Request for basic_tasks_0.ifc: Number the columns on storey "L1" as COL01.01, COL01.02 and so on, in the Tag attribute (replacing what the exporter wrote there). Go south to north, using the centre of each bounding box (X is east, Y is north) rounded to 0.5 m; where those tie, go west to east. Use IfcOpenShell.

First a look at what the model holds.

```python
import ifcopenshell
import ifcopenshell.util.element
import ifcopenshell.util.placement

model = ifcopenshell.open("basic_tasks_0.ifc")
print(model.schema)
storey = next(s for s in model.by_type("IfcBuildingStorey") if s.Name == "L1")
columns = [e for e in ifcopenshell.util.element.get_decomposition(storey) if e.is_a("IfcColumn")]
for e in sorted(columns, key=lambda e: e.id()):
    origin = ifcopenshell.util.placement.get_local_placement(e.ObjectPlacement)[:3, 3]
    print(e.id(), e.Tag, e.Name, origin.round(2) + 0.0, sep=" | ")
```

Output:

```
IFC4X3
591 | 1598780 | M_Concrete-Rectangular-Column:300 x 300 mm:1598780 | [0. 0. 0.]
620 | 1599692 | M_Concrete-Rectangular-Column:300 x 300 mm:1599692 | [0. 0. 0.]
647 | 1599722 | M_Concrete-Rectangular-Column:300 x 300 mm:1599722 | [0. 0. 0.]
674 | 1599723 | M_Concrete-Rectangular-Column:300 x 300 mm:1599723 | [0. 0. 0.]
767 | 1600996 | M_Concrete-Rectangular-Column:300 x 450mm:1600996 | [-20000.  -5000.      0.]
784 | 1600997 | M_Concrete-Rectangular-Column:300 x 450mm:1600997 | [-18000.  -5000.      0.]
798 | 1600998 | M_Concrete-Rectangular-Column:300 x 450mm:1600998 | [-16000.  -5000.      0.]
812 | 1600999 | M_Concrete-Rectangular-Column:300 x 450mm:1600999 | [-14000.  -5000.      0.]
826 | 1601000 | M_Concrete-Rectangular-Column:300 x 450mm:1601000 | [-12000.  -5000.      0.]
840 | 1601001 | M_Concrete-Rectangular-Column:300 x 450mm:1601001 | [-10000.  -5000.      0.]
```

```python
import ifcopenshell
import ifcopenshell.geom
import ifcopenshell.util.element
import ifcopenshell.util.shape

model = ifcopenshell.open("basic_tasks_0.ifc")
settings = ifcopenshell.geom.settings()
settings.set("use-world-coords", True)


def centre(element):
    shape = ifcopenshell.geom.create_shape(settings, element)
    return ifcopenshell.util.shape.get_bbox_centroid(shape.geometry)


storey = next(s for s in model.by_type("IfcBuildingStorey") if s.Name == "L1")
columns = [e for e in ifcopenshell.util.element.get_decomposition(storey) if e.is_a("IfcColumn")]

# Insertion points can sit at a corner or the storey origin, so sort by the geometry (in metres).
centres = {e: centre(e) for e in columns}
columns.sort(key=lambda e: (round(centres[e][1] / 0.5), centres[e][0]))

for i, e in enumerate(columns, start=1):
    number = f"COL01.{i:02d}"
    e.Tag = number
    print(e.id(), number)

model.write("basic_tasks_0_updated.ifc")
```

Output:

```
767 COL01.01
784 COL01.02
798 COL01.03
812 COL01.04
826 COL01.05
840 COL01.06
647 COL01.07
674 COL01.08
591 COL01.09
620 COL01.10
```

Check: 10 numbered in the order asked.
